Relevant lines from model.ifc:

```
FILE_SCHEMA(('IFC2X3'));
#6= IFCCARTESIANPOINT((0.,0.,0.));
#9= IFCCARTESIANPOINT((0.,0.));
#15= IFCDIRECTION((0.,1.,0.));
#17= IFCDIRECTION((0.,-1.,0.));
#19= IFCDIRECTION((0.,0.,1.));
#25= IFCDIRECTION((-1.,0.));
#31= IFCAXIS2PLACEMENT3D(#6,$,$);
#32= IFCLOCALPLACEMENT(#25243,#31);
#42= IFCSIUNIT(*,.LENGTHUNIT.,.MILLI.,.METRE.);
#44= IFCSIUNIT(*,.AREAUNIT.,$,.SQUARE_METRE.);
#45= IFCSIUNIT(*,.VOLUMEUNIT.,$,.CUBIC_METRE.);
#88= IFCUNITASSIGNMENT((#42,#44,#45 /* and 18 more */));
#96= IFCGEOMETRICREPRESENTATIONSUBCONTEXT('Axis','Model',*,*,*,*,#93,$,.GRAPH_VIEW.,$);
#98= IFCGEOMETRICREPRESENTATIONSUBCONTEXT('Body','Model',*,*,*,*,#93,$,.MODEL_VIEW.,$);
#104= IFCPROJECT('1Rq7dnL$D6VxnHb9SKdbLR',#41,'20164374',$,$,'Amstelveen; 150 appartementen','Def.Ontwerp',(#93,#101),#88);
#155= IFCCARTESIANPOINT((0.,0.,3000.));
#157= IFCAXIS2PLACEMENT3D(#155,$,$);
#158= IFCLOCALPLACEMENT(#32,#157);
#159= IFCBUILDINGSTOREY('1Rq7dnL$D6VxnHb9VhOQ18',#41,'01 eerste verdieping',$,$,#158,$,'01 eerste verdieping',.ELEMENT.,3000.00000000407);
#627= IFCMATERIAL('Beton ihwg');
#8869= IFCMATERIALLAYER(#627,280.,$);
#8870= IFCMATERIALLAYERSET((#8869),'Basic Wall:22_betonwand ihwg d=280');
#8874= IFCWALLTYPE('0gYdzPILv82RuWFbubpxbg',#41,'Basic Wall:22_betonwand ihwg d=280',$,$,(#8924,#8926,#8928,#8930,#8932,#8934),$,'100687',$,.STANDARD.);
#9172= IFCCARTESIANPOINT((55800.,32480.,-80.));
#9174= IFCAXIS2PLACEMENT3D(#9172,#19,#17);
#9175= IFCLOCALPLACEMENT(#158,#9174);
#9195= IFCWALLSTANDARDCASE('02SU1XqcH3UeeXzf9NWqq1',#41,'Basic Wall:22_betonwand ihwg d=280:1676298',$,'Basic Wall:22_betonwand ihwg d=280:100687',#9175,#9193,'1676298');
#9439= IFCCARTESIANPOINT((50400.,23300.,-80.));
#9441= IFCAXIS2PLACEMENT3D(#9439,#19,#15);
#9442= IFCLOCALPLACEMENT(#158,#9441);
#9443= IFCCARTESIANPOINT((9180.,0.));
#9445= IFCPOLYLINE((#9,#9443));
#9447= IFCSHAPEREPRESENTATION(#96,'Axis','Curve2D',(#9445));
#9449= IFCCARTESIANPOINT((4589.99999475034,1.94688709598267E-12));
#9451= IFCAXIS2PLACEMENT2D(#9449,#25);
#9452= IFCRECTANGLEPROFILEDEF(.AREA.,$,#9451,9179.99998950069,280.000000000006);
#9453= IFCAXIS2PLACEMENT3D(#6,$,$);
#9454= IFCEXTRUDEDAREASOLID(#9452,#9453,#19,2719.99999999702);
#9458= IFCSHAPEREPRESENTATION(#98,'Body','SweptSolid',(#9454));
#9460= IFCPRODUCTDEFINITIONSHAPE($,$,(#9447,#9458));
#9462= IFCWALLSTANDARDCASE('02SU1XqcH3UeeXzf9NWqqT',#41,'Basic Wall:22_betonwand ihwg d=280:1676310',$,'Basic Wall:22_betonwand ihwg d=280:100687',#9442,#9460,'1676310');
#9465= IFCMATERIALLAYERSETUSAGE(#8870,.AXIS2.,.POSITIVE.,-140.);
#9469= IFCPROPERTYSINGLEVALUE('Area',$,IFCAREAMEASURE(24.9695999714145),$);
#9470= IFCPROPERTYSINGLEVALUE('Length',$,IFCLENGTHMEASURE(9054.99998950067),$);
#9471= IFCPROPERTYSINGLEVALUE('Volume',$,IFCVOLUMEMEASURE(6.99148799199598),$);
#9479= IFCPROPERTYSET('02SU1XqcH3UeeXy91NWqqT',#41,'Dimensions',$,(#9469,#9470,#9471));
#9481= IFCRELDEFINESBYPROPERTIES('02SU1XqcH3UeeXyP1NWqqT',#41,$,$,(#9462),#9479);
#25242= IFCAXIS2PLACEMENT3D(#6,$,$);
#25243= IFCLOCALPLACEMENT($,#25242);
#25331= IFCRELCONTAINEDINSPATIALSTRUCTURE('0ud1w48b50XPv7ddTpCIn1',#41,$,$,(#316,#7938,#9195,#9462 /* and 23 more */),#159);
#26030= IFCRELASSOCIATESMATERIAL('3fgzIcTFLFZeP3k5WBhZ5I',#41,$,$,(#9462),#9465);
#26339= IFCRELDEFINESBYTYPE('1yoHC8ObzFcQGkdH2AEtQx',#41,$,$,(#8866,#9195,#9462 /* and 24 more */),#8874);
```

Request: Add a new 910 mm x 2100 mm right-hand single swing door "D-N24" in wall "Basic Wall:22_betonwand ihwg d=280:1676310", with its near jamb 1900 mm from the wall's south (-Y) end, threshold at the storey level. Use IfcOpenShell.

```python
import numpy as np
import ifcopenshell
import ifcopenshell.api.feature
import ifcopenshell.api.geometry
import ifcopenshell.api.pset
import ifcopenshell.api.root
import ifcopenshell.api.spatial
import ifcopenshell.api.type
import ifcopenshell.geom
import ifcopenshell.util.element
import ifcopenshell.util.placement
import ifcopenshell.util.representation
import ifcopenshell.util.shape
import ifcopenshell.util.unit

model = ifcopenshell.open("model.ifc")
unit_scale = ifcopenshell.util.unit.calculate_unit_scale(model)
area_scale = ifcopenshell.util.unit.calculate_unit_scale(model, "AREAUNIT")
volume_scale = ifcopenshell.util.unit.calculate_unit_scale(model, "VOLUMEUNIT")
settings = ifcopenshell.geom.settings()


def volume(element):
    """Net volume in cubic metres, openings subtracted."""
    shape = ifcopenshell.geom.create_shape(settings, element)
    return ifcopenshell.util.shape.get_volume(shape.geometry)


wall = model.by_guid("02SU1XqcH3UeeXzf9NWqqT")
storey = ifcopenshell.util.element.get_container(wall, ifc_class="IfcBuildingStorey")
context = ifcopenshell.util.representation.get_context(model, "Model", "Body", "MODEL_VIEW")
before = volume(wall)

width, height, from_end, sill = 0.91, 2.1, 1.9, 0.0  # metres

# The wall runs along its own X axis, and the end named is its -X end.
wall_shape = ifcopenshell.geom.create_shape(settings, wall)
x, y, z = ifcopenshell.util.shape.get_vertices(wall_shape.geometry).T
start = x.min() + from_end
face, thickness = float(y.min()), float(y.max() - y.min())
wall_matrix = ifcopenshell.util.placement.get_local_placement(wall.ObjectPlacement)
level = ifcopenshell.util.placement.get_local_placement(storey.ObjectPlacement)[2, 3]


def in_wall(x, y):
    """Placement at x, y metres in the wall's axes, at sill height."""
    matrix = wall_matrix.copy()
    matrix[:, 3] = wall_matrix @ np.array([x / unit_scale, y / unit_scale, 0.0, 1.0])
    matrix[2, 3] = level + sill / unit_scale
    return matrix


# Opening: a box that overshoots both wall faces by 50 mm.
opening = ifcopenshell.api.root.create_entity(model, ifc_class="IfcOpeningElement")
box = ifcopenshell.api.geometry.add_wall_representation(
    model, context=context, length=width, height=height, thickness=thickness + 0.1
)
ifcopenshell.api.geometry.assign_representation(model, product=opening, representation=box)
ifcopenshell.api.geometry.edit_object_placement(model, product=opening, matrix=in_wall(start, face - 0.05), is_si=False)
ifcopenshell.api.feature.add_feature(model, feature=opening, element=wall)

door = ifcopenshell.api.root.create_entity(model, ifc_class="IfcDoor", name="D-N24")
door.OverallWidth, door.OverallHeight = width / unit_scale, height / unit_scale
body = ifcopenshell.api.geometry.add_door_representation(
    model,
    context=context,
    overall_width=door.OverallWidth,
    overall_height=door.OverallHeight,
    operation_type="SINGLE_SWING_RIGHT",
    lining_properties={"LiningDepth": thickness / unit_scale, "ThresholdDepth": thickness / unit_scale},
)
ifcopenshell.api.geometry.assign_representation(model, product=door, representation=body)
ifcopenshell.api.spatial.assign_container(model, products=[door], relating_structure=storey)
fills = ifcopenshell.api.feature.add_filling(model, opening=opening, element=door)
fills.OwnerHistory = door.OwnerHistory  # required in IFC2X3

# IFC2X3 keeps the operation on the door style.
style = ifcopenshell.api.root.create_entity(model, ifc_class="IfcDoorStyle", name="D-N24")
style.OperationType, style.ConstructionType = "SINGLE_SWING_RIGHT", "NOTDEFINED"
style.ParameterTakesPrecedence = style.Sizeable = False
ifcopenshell.api.type.assign_type(model, related_objects=[door], relating_type=style)

# The lining spans the wall, so the door starts at the wall face.
ifcopenshell.api.geometry.edit_object_placement(model, product=door, matrix=in_wall(start, face), is_si=False)

after = volume(wall)

# Update the wall's stored quantities.
pset = model.by_id(ifcopenshell.util.element.get_pset(wall, "Dimensions", should_inherit=False)["id"])
ifcopenshell.api.pset.edit_pset(model, pset=pset, properties={
    "Area": model.create_entity("IfcAreaMeasure", after / thickness / area_scale),
    "Volume": model.create_entity("IfcVolumeMeasure", after / volume_scale),
})

print(f"wall volume {before:.3f} -> {after:.3f} m3")

model.write("model_v2.ifc")
```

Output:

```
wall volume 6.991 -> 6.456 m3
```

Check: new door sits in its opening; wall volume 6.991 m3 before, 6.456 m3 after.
